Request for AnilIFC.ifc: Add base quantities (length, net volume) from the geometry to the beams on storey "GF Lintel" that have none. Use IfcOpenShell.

First a look at what the model holds.

```python
import ifcopenshell
import ifcopenshell.util.element
import ifcopenshell.util.unit

model = ifcopenshell.open("AnilIFC.ifc")
print(model.schema)
for unit_type in ("LENGTHUNIT", "AREAUNIT", "VOLUMEUNIT"):
    print(unit_type, ifcopenshell.util.unit.calculate_unit_scale(model, unit_type))
storey = next(s for s in model.by_type("IfcBuildingStorey") if s.Name == "GF Lintel")
beams = [e for e in ifcopenshell.util.element.get_decomposition(storey) if e.is_a("IfcBeam")]
for e in sorted(beams, key=lambda e: e.id()):
    print(e.id(), e.is_a(), e.Name, list(ifcopenshell.util.element.get_psets(e, qtos_only=True)), sep=" | ")
```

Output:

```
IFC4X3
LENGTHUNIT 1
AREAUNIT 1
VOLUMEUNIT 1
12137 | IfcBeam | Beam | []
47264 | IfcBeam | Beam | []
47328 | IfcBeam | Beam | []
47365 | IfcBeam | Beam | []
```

```python
import ifcopenshell
import ifcopenshell.api.pset
import ifcopenshell.geom
import ifcopenshell.util.element
import ifcopenshell.util.shape
import ifcopenshell.util.unit

model = ifcopenshell.open("AnilIFC.ifc")
unit_scale = ifcopenshell.util.unit.calculate_unit_scale(model)
volume_scale = ifcopenshell.util.unit.calculate_unit_scale(model, "VOLUMEUNIT")
settings = ifcopenshell.geom.settings()

storey = next(s for s in model.by_type("IfcBuildingStorey") if s.Name == "GF Lintel")
beams = [e for e in ifcopenshell.util.element.get_decomposition(storey) if e.is_a("IfcBeam")]

for e in sorted(beams, key=lambda e: e.id()):
    if ifcopenshell.util.element.get_psets(e, qtos_only=True, should_inherit=False):
        continue
    # Geometry comes back in metres, in the element's own axes.
    shape = ifcopenshell.geom.create_shape(settings, e)
    values = {
        "Length": ifcopenshell.util.shape.get_max_xyz(shape.geometry) / unit_scale,
        "NetVolume": ifcopenshell.util.shape.get_volume(shape.geometry) / volume_scale,
    }
    qto = ifcopenshell.api.pset.add_qto(model, product=e, name="Qto_BeamBaseQuantities")
    ifcopenshell.api.pset.edit_qto(model, qto=qto, properties=values)
    print(e.id(), {k: round(v, 3) for k, v in values.items()})

model.write("AnilIFC-out.ifc")
```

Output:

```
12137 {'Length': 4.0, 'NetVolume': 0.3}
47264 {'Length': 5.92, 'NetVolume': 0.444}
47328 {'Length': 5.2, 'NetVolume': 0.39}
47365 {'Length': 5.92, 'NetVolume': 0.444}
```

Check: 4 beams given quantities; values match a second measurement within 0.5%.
